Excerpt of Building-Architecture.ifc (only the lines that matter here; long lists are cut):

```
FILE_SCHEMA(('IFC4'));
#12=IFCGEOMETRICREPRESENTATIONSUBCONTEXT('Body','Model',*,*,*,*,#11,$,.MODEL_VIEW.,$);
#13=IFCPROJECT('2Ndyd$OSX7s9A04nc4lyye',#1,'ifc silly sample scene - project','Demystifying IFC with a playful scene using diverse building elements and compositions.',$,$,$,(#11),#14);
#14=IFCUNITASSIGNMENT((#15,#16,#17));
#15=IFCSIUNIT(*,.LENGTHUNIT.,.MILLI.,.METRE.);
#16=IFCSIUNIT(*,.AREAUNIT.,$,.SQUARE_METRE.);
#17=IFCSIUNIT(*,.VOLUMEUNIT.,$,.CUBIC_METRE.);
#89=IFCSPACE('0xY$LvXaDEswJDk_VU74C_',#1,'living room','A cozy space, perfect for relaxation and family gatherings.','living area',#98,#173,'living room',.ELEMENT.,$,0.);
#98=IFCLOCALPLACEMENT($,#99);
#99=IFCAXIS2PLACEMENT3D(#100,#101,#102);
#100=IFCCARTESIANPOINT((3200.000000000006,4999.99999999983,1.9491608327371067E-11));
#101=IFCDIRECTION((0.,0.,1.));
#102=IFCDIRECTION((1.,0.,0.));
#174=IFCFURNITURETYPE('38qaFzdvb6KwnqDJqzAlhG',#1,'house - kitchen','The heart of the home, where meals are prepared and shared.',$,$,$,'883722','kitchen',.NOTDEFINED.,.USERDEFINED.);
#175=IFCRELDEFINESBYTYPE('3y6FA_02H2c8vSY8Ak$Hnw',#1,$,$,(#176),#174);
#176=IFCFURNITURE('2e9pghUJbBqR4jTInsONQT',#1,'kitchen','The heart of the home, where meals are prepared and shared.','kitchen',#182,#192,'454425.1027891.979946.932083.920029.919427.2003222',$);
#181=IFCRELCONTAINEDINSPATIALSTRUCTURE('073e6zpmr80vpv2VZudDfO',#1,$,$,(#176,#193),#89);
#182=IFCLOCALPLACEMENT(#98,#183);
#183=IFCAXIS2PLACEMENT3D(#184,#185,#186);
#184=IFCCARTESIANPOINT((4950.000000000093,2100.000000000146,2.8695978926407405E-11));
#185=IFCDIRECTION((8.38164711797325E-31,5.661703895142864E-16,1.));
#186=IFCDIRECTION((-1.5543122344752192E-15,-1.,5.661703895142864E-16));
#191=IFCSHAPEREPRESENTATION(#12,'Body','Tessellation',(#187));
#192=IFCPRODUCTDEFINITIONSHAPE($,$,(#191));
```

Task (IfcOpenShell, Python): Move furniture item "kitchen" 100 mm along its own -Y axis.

```python
import ifcopenshell
import ifcopenshell.api.geometry
import ifcopenshell.util.placement

model = ifcopenshell.open("Building-Architecture.ifc")

item = model.by_id(176)
matrix = ifcopenshell.util.placement.get_local_placement(item.ObjectPlacement)
matrix[:3, 3] -= matrix[:3, 1] * 100.0
ifcopenshell.api.geometry.edit_object_placement(model, product=item, matrix=matrix, is_si=False)

print(ifcopenshell.util.placement.get_local_placement(item.ObjectPlacement).round(3) + 0.0)

model.write("Building-Architecture_edited.ifc")
```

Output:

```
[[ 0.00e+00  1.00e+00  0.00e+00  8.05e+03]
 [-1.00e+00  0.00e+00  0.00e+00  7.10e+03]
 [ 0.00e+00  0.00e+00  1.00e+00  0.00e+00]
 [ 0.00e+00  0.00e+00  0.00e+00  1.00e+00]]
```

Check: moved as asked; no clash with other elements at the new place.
